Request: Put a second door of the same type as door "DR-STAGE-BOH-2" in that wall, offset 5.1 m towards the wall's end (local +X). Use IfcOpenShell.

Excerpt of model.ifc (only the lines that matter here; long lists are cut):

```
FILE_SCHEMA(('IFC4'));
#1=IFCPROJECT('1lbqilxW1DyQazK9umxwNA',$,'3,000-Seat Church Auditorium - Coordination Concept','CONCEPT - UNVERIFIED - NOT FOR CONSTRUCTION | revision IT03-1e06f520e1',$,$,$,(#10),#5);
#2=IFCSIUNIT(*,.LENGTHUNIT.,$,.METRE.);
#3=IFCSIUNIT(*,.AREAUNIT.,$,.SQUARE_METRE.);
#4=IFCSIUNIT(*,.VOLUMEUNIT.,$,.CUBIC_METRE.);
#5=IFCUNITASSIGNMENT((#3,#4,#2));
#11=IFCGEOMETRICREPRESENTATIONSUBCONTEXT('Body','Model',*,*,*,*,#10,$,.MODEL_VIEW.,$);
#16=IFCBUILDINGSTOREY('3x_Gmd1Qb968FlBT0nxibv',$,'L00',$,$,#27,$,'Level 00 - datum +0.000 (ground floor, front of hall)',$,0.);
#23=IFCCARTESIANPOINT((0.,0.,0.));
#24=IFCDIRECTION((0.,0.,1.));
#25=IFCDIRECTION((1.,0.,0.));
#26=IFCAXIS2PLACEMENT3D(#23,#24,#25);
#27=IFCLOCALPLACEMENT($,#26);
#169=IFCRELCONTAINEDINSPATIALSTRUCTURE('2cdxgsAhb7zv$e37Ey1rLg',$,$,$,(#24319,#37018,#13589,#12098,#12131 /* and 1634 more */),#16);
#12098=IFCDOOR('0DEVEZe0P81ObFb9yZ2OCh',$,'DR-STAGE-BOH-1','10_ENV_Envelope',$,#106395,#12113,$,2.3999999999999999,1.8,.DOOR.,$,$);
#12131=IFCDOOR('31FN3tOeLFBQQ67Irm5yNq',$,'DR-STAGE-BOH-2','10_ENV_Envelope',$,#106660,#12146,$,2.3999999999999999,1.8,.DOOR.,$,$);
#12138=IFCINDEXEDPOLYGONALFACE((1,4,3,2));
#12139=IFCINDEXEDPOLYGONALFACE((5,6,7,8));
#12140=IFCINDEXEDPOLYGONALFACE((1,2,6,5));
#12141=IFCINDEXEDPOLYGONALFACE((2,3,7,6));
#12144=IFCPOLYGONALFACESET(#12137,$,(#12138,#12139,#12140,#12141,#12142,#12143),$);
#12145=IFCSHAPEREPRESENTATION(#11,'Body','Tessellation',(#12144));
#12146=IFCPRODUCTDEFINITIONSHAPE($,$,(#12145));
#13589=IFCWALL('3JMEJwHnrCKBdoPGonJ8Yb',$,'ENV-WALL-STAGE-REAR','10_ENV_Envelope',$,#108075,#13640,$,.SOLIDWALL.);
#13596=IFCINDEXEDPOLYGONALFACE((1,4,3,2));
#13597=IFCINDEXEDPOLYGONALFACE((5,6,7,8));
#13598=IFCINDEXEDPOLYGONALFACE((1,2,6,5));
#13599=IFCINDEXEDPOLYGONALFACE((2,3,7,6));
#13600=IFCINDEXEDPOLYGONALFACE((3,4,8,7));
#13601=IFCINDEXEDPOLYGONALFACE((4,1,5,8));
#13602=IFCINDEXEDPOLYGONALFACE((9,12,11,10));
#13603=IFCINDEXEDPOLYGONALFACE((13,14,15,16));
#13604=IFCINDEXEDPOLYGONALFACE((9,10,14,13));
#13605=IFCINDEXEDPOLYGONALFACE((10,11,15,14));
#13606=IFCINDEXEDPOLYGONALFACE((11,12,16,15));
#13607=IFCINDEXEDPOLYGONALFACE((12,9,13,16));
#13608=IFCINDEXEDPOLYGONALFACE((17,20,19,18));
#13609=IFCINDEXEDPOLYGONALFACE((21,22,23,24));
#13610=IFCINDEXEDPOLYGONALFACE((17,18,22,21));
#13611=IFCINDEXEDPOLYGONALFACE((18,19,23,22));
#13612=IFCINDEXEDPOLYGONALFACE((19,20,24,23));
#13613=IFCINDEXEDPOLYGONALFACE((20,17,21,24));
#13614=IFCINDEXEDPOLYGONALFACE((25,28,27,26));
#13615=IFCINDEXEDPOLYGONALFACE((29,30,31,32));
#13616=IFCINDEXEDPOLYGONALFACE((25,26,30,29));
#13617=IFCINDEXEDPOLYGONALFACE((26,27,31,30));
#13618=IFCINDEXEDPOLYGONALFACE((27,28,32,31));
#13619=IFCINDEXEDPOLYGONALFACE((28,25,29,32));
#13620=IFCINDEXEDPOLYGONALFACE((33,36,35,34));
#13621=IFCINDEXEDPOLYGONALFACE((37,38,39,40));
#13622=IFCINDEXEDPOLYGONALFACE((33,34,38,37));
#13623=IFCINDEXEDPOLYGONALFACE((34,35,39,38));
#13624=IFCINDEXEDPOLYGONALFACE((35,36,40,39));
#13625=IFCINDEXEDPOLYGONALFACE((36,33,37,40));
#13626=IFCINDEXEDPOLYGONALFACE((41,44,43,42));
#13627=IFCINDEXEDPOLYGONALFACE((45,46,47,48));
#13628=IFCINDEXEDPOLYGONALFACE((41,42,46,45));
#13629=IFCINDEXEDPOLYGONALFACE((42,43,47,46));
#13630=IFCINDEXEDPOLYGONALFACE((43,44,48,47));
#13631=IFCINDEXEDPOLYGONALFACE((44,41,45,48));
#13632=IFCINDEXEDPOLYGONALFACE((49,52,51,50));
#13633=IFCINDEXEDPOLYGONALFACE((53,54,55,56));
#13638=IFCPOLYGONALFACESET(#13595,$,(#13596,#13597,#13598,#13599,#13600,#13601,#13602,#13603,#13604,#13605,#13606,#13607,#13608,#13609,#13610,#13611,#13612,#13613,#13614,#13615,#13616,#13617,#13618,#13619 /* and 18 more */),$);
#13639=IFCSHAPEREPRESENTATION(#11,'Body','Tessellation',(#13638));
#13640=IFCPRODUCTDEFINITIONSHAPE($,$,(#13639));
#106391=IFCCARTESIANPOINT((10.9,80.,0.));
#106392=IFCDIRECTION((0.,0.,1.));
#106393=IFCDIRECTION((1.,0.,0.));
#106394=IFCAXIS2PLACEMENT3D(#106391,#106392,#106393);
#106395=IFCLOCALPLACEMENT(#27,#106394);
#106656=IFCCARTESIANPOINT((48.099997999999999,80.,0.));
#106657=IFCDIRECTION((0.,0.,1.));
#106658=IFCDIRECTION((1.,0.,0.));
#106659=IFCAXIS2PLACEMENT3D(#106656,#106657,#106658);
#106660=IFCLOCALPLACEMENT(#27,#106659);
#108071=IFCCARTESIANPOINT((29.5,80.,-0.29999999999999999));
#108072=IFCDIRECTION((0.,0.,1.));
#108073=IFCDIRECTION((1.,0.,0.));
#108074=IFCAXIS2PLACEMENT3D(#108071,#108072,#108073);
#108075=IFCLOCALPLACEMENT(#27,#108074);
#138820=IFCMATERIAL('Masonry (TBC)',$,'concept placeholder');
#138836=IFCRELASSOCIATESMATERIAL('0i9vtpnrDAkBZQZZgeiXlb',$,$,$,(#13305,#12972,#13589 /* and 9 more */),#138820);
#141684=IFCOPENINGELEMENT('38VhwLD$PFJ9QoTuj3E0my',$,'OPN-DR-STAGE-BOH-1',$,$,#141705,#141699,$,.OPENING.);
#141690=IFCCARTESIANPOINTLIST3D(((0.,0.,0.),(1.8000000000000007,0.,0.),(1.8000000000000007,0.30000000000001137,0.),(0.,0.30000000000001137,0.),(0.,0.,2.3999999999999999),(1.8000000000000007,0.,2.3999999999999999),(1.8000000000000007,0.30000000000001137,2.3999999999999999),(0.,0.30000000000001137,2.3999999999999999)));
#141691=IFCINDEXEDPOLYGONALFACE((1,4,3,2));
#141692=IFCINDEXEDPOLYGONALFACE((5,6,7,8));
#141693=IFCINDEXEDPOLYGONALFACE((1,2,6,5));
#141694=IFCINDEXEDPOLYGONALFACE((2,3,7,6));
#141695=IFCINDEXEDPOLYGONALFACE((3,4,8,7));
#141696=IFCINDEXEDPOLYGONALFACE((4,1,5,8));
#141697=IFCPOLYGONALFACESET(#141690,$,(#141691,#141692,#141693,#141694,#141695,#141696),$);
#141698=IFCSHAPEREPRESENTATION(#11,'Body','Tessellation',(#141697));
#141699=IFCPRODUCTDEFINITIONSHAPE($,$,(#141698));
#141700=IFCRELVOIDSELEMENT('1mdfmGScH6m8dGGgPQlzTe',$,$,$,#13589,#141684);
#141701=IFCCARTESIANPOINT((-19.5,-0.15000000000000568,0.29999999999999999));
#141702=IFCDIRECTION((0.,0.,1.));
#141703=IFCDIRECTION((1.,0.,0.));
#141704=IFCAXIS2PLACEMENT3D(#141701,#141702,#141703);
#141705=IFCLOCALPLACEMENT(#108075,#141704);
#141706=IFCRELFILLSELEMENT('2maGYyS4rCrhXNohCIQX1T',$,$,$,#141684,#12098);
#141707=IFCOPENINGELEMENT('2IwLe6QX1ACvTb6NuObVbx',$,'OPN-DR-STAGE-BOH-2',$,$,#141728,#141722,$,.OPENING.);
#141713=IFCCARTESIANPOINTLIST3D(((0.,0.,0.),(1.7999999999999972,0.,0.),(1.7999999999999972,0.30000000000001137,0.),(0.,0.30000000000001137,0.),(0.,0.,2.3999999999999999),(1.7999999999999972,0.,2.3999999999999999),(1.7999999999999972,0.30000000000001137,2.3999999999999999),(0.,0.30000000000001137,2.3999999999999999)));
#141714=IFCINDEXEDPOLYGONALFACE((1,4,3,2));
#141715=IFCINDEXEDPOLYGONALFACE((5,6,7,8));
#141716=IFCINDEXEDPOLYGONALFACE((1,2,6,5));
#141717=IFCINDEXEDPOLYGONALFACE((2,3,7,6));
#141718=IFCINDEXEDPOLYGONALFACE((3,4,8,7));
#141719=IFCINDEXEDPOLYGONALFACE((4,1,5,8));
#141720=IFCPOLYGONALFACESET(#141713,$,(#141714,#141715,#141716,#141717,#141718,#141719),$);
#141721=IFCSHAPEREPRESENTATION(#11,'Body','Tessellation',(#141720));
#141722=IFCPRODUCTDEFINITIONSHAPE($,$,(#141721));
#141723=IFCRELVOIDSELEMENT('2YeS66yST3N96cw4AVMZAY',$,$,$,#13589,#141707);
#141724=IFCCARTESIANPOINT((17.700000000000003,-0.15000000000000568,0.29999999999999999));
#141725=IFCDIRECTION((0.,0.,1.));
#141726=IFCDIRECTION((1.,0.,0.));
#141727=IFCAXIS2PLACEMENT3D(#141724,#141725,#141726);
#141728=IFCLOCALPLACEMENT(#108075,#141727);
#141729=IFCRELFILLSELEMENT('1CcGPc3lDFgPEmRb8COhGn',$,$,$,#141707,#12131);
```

```python
import ifcopenshell
import ifcopenshell.api.feature
import ifcopenshell.api.geometry
import ifcopenshell.api.root
import ifcopenshell.geom
import ifcopenshell.util.element
import ifcopenshell.util.placement
import ifcopenshell.util.shape
import ifcopenshell.util.unit

model = ifcopenshell.open("model.ifc")
unit_scale = ifcopenshell.util.unit.calculate_unit_scale(model)
settings = ifcopenshell.geom.settings()


def volume(element):
    """Net volume in cubic metres, openings subtracted."""
    shape = ifcopenshell.geom.create_shape(settings, element)
    return ifcopenshell.util.shape.get_volume(shape.geometry)


door = model.by_guid("31FN3tOeLFBQQ67Irm5yNq")
opening = door.FillsVoids[0].RelatingOpeningElement
wall = opening.VoidsElements[0].RelatingBuildingElement
before = volume(wall)
shift = ifcopenshell.util.placement.get_local_placement(wall.ObjectPlacement)[:3, 0] * 5.1 / unit_scale

# copy_class copies the void relationship, type, container and properties, but no geometry.
new_opening = ifcopenshell.api.root.copy_class(model, product=opening)
new_opening.Representation = ifcopenshell.util.element.copy_deep(
    model, opening.Representation, exclude=["IfcGeometricRepresentationContext", "IfcRepresentationMap"]
)
new_door = ifcopenshell.api.root.copy_class(model, product=door)
new_door.Representation = ifcopenshell.util.element.copy_deep(
    model, door.Representation, exclude=["IfcGeometricRepresentationContext", "IfcRepresentationMap"]
)
ifcopenshell.api.feature.add_filling(model, opening=new_opening, element=new_door)

for old, new in ((opening, new_opening), (door, new_door)):
    matrix = ifcopenshell.util.placement.get_local_placement(old.ObjectPlacement)
    matrix[:3, 3] += shift
    ifcopenshell.api.geometry.edit_object_placement(model, product=new, matrix=matrix, is_si=False)

after = volume(wall)

print(f"wall volume {before:.3f} -> {after:.3f} m3")

model.write("model_edited.ifc")
```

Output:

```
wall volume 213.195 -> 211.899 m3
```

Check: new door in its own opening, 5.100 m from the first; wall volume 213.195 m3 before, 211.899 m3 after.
